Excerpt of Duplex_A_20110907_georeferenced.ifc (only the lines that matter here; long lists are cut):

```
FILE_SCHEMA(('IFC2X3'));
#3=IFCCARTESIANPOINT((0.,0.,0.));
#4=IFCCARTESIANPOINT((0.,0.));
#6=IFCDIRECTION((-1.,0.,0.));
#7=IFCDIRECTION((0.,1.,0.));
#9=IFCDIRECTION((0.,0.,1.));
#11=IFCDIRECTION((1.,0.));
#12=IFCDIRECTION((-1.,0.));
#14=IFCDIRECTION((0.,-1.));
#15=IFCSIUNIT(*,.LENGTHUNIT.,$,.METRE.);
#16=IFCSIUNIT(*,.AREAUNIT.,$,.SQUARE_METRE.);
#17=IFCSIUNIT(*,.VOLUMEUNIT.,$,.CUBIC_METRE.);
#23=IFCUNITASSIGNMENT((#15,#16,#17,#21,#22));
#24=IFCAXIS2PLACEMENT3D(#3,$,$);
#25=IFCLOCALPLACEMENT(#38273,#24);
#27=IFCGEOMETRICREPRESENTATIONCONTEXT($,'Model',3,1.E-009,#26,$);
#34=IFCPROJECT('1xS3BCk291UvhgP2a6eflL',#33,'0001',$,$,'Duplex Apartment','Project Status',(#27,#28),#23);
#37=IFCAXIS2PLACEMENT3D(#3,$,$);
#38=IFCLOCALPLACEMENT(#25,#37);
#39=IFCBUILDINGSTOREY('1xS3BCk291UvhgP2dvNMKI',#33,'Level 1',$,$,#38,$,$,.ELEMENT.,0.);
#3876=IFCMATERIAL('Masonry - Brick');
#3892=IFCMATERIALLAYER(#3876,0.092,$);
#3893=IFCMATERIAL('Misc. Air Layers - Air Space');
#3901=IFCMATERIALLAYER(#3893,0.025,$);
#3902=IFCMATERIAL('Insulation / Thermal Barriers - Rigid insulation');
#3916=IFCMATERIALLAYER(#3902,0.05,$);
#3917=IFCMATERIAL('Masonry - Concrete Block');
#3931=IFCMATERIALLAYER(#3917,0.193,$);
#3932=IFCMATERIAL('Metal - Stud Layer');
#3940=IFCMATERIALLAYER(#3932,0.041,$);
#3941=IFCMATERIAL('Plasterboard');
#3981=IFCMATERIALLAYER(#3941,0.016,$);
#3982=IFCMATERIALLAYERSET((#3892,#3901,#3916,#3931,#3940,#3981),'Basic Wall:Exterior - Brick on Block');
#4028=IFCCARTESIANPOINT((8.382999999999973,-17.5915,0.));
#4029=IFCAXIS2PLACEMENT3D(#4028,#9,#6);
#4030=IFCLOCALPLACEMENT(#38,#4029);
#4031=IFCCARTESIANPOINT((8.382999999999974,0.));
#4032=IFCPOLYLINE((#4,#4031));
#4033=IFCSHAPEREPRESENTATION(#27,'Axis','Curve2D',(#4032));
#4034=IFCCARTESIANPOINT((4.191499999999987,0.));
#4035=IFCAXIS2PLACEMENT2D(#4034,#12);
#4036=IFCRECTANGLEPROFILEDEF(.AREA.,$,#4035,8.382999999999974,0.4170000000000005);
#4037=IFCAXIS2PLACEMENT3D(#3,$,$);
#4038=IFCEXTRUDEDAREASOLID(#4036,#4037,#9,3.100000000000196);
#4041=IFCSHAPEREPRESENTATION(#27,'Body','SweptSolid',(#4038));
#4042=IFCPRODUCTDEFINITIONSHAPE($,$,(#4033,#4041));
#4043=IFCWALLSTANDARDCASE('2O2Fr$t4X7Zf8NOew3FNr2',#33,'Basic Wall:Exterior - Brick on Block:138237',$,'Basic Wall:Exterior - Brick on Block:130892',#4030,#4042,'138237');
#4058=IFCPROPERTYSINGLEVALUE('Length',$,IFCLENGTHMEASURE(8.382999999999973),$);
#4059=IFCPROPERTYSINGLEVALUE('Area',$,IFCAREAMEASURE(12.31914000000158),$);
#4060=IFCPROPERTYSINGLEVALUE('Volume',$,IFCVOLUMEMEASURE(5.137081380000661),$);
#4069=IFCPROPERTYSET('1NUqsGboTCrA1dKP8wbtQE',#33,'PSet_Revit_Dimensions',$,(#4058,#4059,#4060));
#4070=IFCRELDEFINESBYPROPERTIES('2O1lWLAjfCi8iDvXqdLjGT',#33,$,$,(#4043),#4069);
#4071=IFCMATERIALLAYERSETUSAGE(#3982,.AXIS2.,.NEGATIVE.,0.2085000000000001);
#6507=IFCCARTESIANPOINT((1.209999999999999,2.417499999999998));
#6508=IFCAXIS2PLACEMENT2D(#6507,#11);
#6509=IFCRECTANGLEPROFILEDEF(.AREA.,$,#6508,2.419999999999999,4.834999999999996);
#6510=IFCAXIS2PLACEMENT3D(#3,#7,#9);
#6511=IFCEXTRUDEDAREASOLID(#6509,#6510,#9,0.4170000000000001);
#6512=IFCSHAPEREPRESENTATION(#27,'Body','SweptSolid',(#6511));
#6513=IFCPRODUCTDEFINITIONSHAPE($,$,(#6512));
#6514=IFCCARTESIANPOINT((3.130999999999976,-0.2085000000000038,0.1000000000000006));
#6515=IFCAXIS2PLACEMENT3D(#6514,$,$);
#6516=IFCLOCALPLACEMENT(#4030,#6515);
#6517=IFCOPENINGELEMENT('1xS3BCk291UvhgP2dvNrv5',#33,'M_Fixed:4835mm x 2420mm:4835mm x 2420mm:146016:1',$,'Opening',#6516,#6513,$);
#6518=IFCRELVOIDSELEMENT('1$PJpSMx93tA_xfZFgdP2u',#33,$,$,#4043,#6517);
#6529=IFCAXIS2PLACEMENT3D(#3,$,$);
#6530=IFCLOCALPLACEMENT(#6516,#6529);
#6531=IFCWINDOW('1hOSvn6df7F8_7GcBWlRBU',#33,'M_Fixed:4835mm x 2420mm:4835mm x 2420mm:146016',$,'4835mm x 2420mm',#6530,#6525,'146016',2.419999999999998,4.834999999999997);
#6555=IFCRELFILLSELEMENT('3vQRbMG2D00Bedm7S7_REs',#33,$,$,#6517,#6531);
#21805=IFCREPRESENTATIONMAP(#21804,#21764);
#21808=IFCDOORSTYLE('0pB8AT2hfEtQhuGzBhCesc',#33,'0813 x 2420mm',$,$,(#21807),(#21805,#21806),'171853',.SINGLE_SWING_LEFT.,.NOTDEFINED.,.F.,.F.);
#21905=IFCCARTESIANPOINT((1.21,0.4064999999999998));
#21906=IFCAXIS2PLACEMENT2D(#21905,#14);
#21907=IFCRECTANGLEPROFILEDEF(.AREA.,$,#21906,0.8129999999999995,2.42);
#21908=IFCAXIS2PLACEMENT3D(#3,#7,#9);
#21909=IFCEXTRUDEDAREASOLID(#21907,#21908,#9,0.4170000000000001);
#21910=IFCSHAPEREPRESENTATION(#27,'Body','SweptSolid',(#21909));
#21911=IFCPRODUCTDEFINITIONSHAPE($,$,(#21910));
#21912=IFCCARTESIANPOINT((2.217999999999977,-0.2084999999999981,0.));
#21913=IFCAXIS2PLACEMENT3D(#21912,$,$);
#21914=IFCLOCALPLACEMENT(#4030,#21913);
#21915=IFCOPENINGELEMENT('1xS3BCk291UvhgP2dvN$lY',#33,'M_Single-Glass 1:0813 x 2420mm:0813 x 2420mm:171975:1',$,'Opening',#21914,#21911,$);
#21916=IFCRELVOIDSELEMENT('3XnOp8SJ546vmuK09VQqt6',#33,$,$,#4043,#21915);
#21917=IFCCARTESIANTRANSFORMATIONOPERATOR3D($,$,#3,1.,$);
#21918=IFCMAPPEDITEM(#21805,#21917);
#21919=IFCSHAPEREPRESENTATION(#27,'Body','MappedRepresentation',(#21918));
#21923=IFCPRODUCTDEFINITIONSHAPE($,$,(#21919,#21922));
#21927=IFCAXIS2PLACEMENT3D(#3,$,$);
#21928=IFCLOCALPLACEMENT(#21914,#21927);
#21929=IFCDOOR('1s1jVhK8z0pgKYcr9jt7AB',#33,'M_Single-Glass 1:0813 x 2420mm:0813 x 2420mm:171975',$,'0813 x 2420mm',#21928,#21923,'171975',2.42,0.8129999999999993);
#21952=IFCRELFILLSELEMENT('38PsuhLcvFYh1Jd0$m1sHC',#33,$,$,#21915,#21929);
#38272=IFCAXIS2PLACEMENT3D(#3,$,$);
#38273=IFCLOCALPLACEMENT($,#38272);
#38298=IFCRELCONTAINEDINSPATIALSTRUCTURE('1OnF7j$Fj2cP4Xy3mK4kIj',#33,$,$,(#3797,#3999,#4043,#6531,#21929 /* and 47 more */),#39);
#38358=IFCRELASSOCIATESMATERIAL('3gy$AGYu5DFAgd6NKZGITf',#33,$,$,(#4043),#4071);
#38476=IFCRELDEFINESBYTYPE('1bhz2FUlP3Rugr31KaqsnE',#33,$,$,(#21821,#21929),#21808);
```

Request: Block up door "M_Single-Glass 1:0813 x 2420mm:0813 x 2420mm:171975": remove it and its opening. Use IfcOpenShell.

```python
import ifcopenshell
import ifcopenshell.api.feature
import ifcopenshell.api.pset
import ifcopenshell.api.root
import ifcopenshell.geom
import ifcopenshell.util.element
import ifcopenshell.util.shape
import ifcopenshell.util.unit

model = ifcopenshell.open("Duplex_A_20110907_georeferenced.ifc")
area_scale = ifcopenshell.util.unit.calculate_unit_scale(model, "AREAUNIT")
volume_scale = ifcopenshell.util.unit.calculate_unit_scale(model, "VOLUMEUNIT")
settings = ifcopenshell.geom.settings()


def volume(element):
    """Net volume in cubic metres, openings subtracted."""
    shape = ifcopenshell.geom.create_shape(settings, element)
    return ifcopenshell.util.shape.get_volume(shape.geometry)


door = model.by_guid("1s1jVhK8z0pgKYcr9jt7AB")
opening = door.FillsVoids[0].RelatingOpeningElement
wall = opening.VoidsElements[0].RelatingBuildingElement
before = volume(wall)

ifcopenshell.api.root.remove_product(model, product=door)
ifcopenshell.api.feature.remove_feature(model, feature=opening)

after = volume(wall)
thickness = 0.417  # wall thickness in metres

# Update the wall's stored quantities.
pset = model.by_id(ifcopenshell.util.element.get_pset(wall, "PSet_Revit_Dimensions", should_inherit=False)["id"])
ifcopenshell.api.pset.edit_pset(model, pset=pset, properties={
    "Area": model.create_entity("IfcAreaMeasure", after / thickness / area_scale),
    "Volume": model.create_entity("IfcVolumeMeasure", after / volume_scale),
})

print(f"wall volume {before:.3f} -> {after:.3f} m3")

model.write("Duplex_A_20110907_georeferenced_rev.ifc")
```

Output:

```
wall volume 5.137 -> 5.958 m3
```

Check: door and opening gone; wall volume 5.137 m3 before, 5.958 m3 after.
